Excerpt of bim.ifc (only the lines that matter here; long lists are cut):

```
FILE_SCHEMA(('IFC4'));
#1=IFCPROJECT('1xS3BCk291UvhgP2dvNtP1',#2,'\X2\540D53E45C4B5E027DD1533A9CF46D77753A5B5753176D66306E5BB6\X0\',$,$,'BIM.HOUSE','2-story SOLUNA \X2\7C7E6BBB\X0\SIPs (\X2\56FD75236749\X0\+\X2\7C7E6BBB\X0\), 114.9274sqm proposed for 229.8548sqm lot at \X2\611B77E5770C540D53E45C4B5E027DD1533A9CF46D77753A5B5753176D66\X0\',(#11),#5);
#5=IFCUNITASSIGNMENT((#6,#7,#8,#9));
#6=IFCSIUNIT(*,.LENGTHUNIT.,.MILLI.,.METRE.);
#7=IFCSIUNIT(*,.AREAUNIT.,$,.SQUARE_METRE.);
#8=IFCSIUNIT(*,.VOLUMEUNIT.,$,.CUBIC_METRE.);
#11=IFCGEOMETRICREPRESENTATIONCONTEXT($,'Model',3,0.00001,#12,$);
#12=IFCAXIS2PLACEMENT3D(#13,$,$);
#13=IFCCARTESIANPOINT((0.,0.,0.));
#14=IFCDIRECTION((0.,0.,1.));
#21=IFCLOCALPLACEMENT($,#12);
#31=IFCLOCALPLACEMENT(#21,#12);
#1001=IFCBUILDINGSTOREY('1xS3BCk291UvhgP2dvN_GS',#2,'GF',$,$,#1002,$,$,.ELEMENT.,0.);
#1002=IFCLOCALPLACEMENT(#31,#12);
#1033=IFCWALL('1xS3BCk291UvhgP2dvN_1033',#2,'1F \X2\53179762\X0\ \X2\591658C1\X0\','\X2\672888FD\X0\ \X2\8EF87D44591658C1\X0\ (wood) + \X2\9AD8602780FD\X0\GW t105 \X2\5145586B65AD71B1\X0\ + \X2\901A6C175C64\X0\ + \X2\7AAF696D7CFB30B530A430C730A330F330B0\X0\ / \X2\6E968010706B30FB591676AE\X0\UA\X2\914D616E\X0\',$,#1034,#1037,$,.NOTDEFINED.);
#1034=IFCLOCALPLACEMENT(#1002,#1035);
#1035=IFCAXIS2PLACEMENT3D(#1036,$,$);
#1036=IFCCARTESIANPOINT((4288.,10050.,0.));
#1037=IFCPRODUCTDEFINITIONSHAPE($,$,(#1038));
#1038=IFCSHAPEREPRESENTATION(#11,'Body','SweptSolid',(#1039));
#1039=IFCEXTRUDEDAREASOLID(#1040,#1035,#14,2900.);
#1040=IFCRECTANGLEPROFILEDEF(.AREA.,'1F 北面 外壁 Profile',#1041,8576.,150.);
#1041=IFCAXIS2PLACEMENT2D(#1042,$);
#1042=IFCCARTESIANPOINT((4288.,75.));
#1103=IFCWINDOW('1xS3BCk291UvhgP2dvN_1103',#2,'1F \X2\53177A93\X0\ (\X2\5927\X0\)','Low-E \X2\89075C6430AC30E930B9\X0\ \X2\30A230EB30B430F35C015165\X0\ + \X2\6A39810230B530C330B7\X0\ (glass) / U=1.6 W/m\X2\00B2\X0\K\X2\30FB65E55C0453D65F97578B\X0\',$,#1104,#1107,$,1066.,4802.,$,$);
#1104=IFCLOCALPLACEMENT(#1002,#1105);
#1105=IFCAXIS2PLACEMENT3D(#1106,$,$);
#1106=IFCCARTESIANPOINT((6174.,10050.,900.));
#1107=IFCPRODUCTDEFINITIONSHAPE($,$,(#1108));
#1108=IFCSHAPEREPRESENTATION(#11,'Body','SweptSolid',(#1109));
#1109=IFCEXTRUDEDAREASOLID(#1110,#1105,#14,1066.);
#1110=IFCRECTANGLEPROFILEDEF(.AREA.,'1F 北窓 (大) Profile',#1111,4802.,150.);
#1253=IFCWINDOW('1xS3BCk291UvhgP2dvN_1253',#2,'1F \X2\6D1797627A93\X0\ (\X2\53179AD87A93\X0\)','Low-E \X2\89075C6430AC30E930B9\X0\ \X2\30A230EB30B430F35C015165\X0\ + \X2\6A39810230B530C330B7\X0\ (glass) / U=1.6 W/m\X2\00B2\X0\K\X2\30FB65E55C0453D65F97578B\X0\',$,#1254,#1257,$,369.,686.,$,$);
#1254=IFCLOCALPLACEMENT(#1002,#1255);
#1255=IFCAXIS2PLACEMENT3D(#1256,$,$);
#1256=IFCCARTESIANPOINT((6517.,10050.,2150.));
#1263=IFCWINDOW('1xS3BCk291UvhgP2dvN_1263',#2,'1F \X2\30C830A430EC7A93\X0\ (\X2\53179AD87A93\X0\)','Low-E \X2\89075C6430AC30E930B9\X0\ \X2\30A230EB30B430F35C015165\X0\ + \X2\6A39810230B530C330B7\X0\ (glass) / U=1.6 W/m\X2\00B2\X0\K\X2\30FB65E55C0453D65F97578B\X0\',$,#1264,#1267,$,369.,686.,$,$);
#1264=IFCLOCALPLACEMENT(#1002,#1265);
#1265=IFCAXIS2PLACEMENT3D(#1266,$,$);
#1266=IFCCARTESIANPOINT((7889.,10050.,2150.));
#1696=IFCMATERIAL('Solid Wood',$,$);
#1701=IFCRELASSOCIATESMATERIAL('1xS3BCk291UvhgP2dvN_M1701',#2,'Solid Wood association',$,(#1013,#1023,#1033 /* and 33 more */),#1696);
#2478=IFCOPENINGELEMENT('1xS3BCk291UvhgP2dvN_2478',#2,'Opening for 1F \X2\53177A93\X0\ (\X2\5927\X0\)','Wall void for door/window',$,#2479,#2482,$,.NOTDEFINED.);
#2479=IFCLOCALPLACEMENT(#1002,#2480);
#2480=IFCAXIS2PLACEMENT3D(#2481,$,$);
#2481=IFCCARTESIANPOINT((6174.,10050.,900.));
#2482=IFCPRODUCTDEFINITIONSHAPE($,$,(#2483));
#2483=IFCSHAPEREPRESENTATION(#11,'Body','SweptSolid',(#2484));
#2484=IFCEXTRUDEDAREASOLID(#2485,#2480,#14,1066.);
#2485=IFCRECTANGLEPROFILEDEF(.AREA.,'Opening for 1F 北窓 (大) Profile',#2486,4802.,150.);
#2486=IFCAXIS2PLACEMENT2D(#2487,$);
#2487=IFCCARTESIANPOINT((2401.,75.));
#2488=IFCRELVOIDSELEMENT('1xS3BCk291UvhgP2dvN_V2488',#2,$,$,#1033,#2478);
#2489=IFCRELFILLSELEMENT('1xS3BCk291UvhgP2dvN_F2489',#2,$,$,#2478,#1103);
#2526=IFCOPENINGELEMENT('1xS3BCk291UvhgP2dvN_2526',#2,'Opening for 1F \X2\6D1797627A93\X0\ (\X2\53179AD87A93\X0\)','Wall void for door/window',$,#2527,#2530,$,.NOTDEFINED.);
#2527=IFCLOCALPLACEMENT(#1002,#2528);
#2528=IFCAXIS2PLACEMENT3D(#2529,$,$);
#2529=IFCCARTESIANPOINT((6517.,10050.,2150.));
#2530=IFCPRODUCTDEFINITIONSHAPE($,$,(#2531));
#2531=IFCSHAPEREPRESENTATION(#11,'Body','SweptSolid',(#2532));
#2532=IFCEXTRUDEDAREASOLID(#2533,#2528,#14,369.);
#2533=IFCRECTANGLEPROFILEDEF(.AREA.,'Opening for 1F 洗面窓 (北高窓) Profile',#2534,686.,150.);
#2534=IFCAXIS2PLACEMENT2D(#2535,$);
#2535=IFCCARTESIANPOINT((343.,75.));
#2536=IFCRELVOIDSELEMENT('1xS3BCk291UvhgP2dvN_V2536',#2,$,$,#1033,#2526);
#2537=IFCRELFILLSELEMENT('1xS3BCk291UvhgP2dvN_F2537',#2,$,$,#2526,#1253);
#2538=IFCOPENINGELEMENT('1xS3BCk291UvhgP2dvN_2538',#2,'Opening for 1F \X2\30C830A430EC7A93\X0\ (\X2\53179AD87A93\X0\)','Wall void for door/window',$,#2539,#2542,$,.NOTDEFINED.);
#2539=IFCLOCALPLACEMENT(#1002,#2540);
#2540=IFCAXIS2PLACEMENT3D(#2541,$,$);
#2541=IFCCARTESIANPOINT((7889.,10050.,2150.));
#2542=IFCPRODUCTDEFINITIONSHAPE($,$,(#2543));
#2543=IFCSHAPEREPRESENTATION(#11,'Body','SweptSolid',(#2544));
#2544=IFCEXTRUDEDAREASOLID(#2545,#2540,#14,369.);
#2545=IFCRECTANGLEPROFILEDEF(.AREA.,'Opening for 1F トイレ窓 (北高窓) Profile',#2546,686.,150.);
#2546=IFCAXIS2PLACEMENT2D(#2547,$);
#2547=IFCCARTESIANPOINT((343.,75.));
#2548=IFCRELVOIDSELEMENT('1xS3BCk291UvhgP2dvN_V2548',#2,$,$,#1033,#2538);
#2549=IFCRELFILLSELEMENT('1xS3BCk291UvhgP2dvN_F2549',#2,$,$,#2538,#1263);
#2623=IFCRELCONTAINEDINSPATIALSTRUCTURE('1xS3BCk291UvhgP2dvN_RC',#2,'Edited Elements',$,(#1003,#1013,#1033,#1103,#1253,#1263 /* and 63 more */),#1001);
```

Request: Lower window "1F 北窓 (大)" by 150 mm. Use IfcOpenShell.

```python
import numpy as np
import ifcopenshell
import ifcopenshell.api.geometry
import ifcopenshell.util.placement
import ifcopenshell.util.unit

model = ifcopenshell.open("bim.ifc")
unit_scale = ifcopenshell.util.unit.calculate_unit_scale(model)

window = model.by_guid("1xS3BCk291UvhgP2dvN_1103")
opening = window.FillsVoids[0].RelatingOpeningElement
dz = -0.15 / unit_scale

shift = np.array([0.0, 0.0, dz])
# The window is not placed relative to its opening, so move both.
for product in (opening, window):
    matrix = ifcopenshell.util.placement.get_local_placement(product.ObjectPlacement)
    matrix[:3, 3] += shift
    ifcopenshell.api.geometry.edit_object_placement(model, product=product, matrix=matrix, is_si=False)

print(f"moved by {dz * unit_scale:+.3f} m")

model.write("bim_rev.ifc")
```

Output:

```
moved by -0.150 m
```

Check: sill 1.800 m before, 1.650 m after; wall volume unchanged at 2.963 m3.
